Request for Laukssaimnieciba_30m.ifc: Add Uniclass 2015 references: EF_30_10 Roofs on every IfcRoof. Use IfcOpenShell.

First a look at what the model holds.

```python
import ifcopenshell

model = ifcopenshell.open("Laukssaimnieciba_30m.ifc")
print(model.schema)
print("classifications:", [c.Name for c in model.by_type("IfcClassification")])
for ifc_class in ("IfcDoor", "IfcRoof", "IfcStair", "IfcWall", "IfcWindow"):
    print(ifc_class, len(model.by_type(ifc_class)))
```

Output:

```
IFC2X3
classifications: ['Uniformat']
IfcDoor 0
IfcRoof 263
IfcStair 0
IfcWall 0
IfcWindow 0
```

```python
import ifcopenshell
import ifcopenshell.api.classification

model = ifcopenshell.open("Laukssaimnieciba_30m.ifc")

# IFC2X3 requires Source and Edition and has no link from the project to the system.
system = model.create_entity("IfcClassification", Source="NBS", Edition="2015", Name="Uniclass 2015")

codes = {
    "IfcRoof": ("EF_30_10", "Roofs"),
}
for ifc_class, (code, name) in codes.items():
    products = model.by_type(ifc_class)
    ifcopenshell.api.classification.add_reference(
        model, products=products, classification=system, identification=code, name=name
    )
    print(code, len(products))

model.write("Laukssaimnieciba_30m_edited.ifc")
```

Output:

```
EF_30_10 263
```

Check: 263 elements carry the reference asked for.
